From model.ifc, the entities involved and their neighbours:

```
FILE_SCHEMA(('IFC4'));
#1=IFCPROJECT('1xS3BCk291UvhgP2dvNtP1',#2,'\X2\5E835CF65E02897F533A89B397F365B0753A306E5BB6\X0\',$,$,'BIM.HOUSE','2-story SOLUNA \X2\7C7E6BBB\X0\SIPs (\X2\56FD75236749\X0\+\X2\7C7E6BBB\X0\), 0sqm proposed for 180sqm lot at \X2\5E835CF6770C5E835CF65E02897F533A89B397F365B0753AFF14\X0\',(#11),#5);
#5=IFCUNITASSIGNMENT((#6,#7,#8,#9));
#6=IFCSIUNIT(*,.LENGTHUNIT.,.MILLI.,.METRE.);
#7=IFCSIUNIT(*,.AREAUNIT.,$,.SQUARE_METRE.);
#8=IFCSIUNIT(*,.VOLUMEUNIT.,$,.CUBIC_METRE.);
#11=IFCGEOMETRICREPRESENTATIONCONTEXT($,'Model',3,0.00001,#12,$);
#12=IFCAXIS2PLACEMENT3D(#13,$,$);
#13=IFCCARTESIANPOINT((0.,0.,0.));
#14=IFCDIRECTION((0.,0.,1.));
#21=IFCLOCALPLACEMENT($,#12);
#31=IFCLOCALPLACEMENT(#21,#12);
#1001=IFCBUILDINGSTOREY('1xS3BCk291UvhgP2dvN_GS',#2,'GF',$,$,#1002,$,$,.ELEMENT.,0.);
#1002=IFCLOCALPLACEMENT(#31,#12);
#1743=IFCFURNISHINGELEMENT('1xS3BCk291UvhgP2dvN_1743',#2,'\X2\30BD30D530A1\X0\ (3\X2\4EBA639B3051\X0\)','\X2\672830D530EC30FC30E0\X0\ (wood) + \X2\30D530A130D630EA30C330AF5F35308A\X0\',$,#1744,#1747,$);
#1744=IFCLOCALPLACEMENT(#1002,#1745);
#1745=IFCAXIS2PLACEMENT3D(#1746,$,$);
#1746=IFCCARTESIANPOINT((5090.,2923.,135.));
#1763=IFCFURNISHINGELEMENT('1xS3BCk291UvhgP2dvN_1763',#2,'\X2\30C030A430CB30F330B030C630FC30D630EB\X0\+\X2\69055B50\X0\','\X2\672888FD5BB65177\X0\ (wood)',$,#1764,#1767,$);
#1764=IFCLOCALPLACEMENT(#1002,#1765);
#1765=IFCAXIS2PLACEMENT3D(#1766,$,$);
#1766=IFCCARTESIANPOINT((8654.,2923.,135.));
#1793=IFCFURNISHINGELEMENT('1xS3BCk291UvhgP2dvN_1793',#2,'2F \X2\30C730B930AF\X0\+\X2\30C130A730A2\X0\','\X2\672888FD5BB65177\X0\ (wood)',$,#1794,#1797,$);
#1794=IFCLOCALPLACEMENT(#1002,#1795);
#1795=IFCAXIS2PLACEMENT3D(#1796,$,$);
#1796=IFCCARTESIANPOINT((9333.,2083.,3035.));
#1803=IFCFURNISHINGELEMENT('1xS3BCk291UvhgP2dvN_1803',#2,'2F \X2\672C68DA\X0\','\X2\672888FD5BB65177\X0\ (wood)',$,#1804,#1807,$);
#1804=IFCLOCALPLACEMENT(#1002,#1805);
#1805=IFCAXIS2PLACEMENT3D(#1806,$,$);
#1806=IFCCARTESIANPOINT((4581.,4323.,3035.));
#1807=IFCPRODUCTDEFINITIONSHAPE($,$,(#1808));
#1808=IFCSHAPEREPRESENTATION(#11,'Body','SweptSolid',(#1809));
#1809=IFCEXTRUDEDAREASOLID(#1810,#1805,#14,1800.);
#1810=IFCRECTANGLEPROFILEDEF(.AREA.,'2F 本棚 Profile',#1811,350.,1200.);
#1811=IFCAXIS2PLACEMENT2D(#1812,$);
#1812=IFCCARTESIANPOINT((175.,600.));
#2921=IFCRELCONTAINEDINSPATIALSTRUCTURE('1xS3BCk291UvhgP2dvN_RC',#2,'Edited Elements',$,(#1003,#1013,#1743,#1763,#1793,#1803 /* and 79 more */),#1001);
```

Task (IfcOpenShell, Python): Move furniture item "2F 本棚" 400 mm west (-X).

```python
import ifcopenshell
import ifcopenshell.api.geometry
import ifcopenshell.util.placement

model = ifcopenshell.open("model.ifc")

item = model.by_guid("1xS3BCk291UvhgP2dvN_1803")
matrix = ifcopenshell.util.placement.get_local_placement(item.ObjectPlacement)
matrix[0, 3] -= 400.0
ifcopenshell.api.geometry.edit_object_placement(model, product=item, matrix=matrix, is_si=False)

print(ifcopenshell.util.placement.get_local_placement(item.ObjectPlacement).round(3) + 0.0)

model.write("model_v2.ifc")
```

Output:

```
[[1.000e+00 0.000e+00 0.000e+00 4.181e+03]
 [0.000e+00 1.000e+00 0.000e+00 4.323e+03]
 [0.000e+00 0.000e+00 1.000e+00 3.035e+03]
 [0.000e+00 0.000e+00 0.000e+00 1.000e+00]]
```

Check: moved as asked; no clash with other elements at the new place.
